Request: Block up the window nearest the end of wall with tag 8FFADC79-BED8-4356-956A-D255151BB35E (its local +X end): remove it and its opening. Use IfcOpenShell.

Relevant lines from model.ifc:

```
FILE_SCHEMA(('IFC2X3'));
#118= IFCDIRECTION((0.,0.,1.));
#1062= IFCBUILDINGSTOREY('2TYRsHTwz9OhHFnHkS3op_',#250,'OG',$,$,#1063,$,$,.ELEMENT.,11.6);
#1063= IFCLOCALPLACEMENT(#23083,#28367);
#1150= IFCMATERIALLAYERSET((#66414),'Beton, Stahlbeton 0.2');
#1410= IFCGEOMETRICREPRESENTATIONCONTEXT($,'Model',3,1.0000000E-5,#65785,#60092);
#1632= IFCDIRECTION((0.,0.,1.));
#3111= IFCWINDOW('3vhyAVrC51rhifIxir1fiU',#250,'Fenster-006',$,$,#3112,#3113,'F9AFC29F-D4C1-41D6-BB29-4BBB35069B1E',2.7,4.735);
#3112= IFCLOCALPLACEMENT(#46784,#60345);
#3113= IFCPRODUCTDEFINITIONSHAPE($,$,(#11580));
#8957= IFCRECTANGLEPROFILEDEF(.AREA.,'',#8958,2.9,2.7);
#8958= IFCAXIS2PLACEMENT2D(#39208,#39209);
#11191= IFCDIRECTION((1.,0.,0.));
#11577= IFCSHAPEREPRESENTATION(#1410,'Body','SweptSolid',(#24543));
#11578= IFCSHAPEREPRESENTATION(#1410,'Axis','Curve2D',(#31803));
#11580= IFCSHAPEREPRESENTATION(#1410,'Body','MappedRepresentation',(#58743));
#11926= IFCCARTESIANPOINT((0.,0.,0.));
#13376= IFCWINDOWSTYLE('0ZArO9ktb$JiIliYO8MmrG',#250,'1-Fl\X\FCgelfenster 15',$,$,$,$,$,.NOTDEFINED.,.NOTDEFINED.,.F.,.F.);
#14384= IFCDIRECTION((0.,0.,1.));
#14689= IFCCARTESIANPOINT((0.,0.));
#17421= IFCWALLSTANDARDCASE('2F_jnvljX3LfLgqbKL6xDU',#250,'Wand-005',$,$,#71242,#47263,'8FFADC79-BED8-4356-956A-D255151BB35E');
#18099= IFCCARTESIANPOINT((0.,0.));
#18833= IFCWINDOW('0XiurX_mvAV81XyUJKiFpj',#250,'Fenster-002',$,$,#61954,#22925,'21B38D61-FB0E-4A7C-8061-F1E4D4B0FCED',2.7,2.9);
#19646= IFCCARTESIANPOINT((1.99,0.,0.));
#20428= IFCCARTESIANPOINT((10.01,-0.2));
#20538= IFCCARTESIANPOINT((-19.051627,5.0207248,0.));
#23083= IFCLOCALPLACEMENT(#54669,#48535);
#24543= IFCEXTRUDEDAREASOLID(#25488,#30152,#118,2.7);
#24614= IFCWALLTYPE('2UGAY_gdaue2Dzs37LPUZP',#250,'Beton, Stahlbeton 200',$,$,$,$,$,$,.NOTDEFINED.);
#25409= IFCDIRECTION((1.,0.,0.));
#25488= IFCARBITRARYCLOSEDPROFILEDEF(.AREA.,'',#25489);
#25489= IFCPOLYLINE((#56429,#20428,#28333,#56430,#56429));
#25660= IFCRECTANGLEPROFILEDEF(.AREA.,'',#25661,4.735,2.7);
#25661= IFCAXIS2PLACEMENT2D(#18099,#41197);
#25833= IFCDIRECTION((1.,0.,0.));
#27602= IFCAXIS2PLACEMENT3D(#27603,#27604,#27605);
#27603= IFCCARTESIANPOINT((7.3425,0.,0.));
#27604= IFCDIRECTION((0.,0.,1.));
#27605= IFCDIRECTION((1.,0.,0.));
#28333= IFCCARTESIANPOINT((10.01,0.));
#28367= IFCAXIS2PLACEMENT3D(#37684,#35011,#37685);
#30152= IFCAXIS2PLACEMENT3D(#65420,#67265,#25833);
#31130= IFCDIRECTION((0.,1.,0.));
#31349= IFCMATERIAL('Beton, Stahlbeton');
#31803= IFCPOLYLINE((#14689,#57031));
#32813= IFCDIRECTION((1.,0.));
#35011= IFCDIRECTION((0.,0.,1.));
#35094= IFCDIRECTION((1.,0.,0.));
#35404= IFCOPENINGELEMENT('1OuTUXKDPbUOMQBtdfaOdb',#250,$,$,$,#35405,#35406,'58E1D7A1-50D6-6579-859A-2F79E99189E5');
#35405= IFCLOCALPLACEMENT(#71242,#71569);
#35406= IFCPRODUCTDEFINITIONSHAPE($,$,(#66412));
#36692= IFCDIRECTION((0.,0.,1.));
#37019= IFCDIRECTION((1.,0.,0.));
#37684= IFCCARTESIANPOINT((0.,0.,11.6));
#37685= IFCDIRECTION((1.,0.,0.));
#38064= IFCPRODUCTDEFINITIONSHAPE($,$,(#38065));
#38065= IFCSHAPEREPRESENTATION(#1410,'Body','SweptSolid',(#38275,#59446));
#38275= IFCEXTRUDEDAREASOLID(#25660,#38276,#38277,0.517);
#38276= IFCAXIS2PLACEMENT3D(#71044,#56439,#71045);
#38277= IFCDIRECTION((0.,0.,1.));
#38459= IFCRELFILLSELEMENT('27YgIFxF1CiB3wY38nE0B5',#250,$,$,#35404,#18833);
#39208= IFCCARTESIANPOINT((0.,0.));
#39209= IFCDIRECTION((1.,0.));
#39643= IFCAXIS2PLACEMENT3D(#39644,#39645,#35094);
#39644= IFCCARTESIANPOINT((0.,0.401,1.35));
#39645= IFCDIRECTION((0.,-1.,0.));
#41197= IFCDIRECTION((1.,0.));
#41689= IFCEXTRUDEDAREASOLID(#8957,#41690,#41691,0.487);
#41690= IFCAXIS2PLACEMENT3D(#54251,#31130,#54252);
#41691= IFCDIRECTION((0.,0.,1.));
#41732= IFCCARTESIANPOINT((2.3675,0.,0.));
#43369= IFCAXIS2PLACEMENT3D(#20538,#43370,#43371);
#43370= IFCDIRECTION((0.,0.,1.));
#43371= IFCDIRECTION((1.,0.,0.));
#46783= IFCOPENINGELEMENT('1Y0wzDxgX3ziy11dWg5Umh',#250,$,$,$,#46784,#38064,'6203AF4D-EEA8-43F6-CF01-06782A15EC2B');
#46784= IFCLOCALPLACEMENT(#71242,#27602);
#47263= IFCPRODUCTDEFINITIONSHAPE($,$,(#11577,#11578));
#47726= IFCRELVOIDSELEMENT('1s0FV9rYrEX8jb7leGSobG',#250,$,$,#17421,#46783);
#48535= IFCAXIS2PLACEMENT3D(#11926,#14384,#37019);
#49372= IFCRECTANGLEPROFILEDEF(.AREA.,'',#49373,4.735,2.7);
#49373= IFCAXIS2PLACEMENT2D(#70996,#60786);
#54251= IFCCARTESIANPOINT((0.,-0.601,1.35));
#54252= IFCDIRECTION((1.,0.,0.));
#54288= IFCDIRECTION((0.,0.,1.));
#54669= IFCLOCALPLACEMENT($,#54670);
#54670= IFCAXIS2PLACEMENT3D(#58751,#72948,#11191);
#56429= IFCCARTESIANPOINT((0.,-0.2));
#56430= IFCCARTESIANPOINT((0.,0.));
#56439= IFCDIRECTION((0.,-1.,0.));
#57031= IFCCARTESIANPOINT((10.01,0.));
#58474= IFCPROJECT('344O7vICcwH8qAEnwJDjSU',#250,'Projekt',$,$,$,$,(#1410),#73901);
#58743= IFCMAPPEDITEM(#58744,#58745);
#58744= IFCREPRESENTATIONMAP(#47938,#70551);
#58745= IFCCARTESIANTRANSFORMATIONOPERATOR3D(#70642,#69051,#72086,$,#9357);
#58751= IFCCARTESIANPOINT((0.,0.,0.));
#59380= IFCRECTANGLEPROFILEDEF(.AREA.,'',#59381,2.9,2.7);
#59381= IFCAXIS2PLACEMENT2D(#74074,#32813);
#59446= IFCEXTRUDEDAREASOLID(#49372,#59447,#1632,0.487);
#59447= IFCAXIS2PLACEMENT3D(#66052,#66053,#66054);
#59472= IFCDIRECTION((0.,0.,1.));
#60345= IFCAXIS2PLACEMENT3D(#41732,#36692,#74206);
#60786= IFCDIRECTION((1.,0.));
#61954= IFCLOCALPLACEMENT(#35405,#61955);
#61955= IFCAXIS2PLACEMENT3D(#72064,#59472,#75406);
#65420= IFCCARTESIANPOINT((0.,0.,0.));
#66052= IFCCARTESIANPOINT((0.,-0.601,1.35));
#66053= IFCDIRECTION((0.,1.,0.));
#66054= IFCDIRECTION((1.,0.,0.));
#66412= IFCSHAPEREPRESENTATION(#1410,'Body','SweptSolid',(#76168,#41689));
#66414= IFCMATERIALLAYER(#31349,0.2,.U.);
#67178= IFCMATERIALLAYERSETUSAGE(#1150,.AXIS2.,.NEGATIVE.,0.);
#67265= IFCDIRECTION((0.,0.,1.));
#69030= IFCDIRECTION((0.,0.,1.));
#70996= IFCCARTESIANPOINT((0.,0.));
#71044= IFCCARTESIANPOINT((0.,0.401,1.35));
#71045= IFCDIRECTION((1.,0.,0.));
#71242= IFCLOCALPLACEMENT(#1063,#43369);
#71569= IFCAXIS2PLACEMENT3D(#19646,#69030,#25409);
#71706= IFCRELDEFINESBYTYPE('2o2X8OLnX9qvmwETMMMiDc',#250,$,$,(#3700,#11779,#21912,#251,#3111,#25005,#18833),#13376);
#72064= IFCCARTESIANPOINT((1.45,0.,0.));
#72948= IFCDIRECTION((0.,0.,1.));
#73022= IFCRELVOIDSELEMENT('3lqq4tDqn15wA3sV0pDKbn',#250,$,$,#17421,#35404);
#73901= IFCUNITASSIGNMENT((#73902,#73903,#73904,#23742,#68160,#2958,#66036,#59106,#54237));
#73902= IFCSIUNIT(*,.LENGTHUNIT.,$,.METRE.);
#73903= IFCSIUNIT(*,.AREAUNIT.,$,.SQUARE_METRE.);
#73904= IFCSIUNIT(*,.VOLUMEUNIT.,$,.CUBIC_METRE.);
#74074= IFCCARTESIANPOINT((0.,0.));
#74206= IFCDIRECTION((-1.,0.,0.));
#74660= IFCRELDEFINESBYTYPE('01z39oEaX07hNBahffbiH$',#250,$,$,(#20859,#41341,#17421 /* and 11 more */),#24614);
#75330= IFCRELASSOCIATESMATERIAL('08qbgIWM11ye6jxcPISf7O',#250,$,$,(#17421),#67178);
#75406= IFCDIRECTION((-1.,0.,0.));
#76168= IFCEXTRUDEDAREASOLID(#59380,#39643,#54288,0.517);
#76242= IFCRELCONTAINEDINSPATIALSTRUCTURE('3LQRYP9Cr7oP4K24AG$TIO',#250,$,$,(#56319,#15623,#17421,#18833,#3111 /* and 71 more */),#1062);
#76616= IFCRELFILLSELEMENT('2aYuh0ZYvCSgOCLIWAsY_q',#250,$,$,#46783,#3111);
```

```python
import ifcopenshell
import ifcopenshell.api.feature
import ifcopenshell.api.root
import ifcopenshell.geom
import ifcopenshell.util.shape

model = ifcopenshell.open("model.ifc")
settings = ifcopenshell.geom.settings()


def volume(element):
    """Net volume in cubic metres, openings subtracted."""
    shape = ifcopenshell.geom.create_shape(settings, element)
    return ifcopenshell.util.shape.get_volume(shape.geometry)


window = model.by_id(3111)
opening = window.FillsVoids[0].RelatingOpeningElement
wall = opening.VoidsElements[0].RelatingBuildingElement
before = volume(wall)

ifcopenshell.api.root.remove_product(model, product=window)
ifcopenshell.api.feature.remove_feature(model, feature=opening)

after = volume(wall)

print(f"wall volume {before:.3f} -> {after:.3f} m3")

model.write("model_edited.ifc")
```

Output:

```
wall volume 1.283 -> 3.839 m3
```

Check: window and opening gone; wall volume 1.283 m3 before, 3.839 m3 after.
